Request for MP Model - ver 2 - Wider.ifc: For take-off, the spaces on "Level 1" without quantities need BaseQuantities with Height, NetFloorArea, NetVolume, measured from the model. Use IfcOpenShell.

First a look at what the model holds.

```python
import ifcopenshell
import ifcopenshell.util.element
import ifcopenshell.util.unit

model = ifcopenshell.open("MP Model - ver 2 - Wider.ifc")
print(model.schema)
for unit_type in ("LENGTHUNIT", "AREAUNIT", "VOLUMEUNIT"):
    print(unit_type, ifcopenshell.util.unit.calculate_unit_scale(model, unit_type))
storey = next(s for s in model.by_type("IfcBuildingStorey") if s.Name == "Level 1")
spaces = [e for e in ifcopenshell.util.element.get_decomposition(storey) if e.is_a("IfcSpace")]
for e in sorted(spaces, key=lambda e: e.id()):
    print(e.id(), e.is_a(), e.Name, list(ifcopenshell.util.element.get_psets(e, qtos_only=True)), sep=" | ")
```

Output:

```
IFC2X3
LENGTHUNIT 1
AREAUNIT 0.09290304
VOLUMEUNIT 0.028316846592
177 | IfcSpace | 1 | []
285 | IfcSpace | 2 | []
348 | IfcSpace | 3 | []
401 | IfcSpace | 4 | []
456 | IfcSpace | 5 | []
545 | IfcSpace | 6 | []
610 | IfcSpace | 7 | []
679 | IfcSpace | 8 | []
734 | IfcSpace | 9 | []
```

```python
import ifcopenshell
import ifcopenshell.api.pset
import ifcopenshell.geom
import ifcopenshell.util.element
import ifcopenshell.util.shape
import ifcopenshell.util.unit

model = ifcopenshell.open("MP Model - ver 2 - Wider.ifc")
unit_scale = ifcopenshell.util.unit.calculate_unit_scale(model)
area_scale = ifcopenshell.util.unit.calculate_unit_scale(model, "AREAUNIT")
volume_scale = ifcopenshell.util.unit.calculate_unit_scale(model, "VOLUMEUNIT")
settings = ifcopenshell.geom.settings()

storey = next(s for s in model.by_type("IfcBuildingStorey") if s.Name == "Level 1")
spaces = [e for e in ifcopenshell.util.element.get_decomposition(storey) if e.is_a("IfcSpace")]

for e in sorted(spaces, key=lambda e: e.id()):
    if ifcopenshell.util.element.get_psets(e, qtos_only=True, should_inherit=False):
        continue
    # Geometry comes back in metres, in the element's own axes.
    shape = ifcopenshell.geom.create_shape(settings, e)
    values = {
        "Height": ifcopenshell.util.shape.get_z(shape.geometry) / unit_scale,
        "NetFloorArea": ifcopenshell.util.shape.get_footprint_area(shape.geometry) / area_scale,
        "NetVolume": ifcopenshell.util.shape.get_volume(shape.geometry) / volume_scale,
    }
    qto = ifcopenshell.api.pset.add_qto(model, product=e, name="BaseQuantities")
    ifcopenshell.api.pset.edit_qto(model, qto=qto, properties=values)
    print(e.id(), {k: round(v, 3) for k, v in values.items()})

model.write("MP Model - ver 2 - Wider_v2.ifc")
```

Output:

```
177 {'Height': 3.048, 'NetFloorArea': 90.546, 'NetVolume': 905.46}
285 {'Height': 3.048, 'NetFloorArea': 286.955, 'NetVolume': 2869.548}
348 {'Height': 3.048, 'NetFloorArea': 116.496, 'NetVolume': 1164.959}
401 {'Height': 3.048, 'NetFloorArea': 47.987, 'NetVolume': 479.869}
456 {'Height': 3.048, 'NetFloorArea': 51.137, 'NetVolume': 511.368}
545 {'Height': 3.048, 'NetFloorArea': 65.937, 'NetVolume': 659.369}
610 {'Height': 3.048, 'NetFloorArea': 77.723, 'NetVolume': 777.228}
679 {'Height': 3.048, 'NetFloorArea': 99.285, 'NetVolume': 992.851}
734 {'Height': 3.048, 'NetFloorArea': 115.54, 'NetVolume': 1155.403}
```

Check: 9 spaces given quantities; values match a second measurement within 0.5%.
